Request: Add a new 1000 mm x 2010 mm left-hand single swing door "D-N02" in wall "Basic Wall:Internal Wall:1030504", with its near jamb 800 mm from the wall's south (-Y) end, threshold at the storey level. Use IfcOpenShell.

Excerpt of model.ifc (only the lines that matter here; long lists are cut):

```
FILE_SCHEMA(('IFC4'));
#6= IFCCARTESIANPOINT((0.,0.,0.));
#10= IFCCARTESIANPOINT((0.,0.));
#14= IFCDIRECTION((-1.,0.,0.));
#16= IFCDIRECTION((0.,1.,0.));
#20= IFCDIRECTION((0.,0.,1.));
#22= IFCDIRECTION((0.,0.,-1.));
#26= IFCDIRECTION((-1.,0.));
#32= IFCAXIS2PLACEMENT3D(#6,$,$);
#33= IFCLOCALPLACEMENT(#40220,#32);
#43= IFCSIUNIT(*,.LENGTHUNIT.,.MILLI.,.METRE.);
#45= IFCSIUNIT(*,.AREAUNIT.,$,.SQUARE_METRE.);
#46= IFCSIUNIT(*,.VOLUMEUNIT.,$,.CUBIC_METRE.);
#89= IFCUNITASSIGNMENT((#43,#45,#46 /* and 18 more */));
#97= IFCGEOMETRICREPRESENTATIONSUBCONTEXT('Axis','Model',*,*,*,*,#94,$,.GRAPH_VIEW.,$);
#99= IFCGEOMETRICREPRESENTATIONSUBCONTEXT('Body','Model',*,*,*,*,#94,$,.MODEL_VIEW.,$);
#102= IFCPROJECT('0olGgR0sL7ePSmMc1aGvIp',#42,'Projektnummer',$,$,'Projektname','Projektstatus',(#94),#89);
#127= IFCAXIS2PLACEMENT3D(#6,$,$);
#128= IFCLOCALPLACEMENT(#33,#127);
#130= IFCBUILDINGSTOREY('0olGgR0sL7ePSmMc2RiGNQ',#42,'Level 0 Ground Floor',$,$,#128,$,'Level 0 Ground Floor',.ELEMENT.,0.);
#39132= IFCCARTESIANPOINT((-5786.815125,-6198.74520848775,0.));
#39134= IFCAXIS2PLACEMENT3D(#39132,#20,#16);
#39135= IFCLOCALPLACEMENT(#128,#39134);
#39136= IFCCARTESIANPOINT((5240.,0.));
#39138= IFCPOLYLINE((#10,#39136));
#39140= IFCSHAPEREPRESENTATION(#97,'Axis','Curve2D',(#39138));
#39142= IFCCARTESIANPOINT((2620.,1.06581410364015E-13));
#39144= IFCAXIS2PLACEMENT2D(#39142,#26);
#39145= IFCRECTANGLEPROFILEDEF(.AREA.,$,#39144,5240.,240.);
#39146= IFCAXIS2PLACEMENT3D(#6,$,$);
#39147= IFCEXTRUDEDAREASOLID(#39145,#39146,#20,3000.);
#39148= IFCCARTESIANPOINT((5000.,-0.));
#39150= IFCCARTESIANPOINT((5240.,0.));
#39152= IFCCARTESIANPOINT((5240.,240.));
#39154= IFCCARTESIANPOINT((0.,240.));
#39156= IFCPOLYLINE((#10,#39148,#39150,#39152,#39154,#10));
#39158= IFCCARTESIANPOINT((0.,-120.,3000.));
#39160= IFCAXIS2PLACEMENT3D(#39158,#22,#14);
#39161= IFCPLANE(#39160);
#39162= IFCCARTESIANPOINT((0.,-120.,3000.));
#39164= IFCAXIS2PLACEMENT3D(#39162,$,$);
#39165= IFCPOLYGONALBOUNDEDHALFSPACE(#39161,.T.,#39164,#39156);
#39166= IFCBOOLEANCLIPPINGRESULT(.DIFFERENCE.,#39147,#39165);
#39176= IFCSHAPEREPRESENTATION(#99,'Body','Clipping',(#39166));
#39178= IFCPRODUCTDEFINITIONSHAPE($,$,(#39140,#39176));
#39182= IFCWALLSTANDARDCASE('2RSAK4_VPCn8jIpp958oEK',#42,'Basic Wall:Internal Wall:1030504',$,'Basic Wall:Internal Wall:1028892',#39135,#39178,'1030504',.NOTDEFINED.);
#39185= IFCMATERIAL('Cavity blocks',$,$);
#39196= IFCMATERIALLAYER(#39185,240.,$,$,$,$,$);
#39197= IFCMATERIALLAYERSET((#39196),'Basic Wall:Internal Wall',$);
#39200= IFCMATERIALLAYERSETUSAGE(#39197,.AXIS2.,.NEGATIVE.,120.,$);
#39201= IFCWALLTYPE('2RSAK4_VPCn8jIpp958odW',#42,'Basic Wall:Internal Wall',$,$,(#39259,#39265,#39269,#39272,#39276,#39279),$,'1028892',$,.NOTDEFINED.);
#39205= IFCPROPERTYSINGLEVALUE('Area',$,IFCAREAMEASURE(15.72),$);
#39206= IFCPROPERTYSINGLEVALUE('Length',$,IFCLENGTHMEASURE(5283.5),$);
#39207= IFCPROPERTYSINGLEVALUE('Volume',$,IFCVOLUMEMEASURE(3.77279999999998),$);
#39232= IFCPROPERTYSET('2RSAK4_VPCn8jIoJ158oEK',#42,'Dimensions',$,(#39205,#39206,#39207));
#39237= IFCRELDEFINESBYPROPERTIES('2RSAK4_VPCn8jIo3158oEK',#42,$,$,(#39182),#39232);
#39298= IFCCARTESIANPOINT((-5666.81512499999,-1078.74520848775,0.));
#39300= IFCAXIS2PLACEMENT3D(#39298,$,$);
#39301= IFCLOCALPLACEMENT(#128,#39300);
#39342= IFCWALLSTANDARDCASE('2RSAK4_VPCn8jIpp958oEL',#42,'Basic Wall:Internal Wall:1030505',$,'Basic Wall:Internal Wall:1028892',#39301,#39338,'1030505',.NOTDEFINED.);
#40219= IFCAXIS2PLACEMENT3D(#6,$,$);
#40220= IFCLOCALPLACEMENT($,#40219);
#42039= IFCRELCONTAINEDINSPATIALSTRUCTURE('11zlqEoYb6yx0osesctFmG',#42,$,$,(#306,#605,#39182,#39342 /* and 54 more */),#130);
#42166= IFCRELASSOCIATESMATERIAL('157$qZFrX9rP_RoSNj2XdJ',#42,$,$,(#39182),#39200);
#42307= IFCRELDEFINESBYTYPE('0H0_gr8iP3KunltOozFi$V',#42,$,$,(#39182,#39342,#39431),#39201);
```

```python
import numpy as np
import ifcopenshell
import ifcopenshell.api.feature
import ifcopenshell.api.geometry
import ifcopenshell.api.pset
import ifcopenshell.api.root
import ifcopenshell.api.spatial
import ifcopenshell.geom
import ifcopenshell.util.element
import ifcopenshell.util.placement
import ifcopenshell.util.representation
import ifcopenshell.util.shape
import ifcopenshell.util.unit

model = ifcopenshell.open("model.ifc")
unit_scale = ifcopenshell.util.unit.calculate_unit_scale(model)
area_scale = ifcopenshell.util.unit.calculate_unit_scale(model, "AREAUNIT")
volume_scale = ifcopenshell.util.unit.calculate_unit_scale(model, "VOLUMEUNIT")
settings = ifcopenshell.geom.settings()


def volume(element):
    """Net volume in cubic metres, openings subtracted."""
    shape = ifcopenshell.geom.create_shape(settings, element)
    return ifcopenshell.util.shape.get_volume(shape.geometry)


wall = model.by_guid("2RSAK4_VPCn8jIpp958oEK")
storey = ifcopenshell.util.element.get_container(wall, ifc_class="IfcBuildingStorey")
context = ifcopenshell.util.representation.get_context(model, "Model", "Body", "MODEL_VIEW")
before = volume(wall)

width, height, from_end, sill = 1, 2.01, 0.8, 0.0  # metres

# The wall runs along its own X axis, and the end named is its -X end.
wall_shape = ifcopenshell.geom.create_shape(settings, wall)
x, y, z = ifcopenshell.util.shape.get_vertices(wall_shape.geometry).T
start = x.min() + from_end
face, thickness = float(y.min()), float(y.max() - y.min())
wall_matrix = ifcopenshell.util.placement.get_local_placement(wall.ObjectPlacement)
level = ifcopenshell.util.placement.get_local_placement(storey.ObjectPlacement)[2, 3]


def in_wall(x, y):
    """Placement at x, y metres in the wall's axes, at sill height."""
    matrix = wall_matrix.copy()
    matrix[:, 3] = wall_matrix @ np.array([x / unit_scale, y / unit_scale, 0.0, 1.0])
    matrix[2, 3] = level + sill / unit_scale
    return matrix


# Opening: a box that overshoots both wall faces by 50 mm.
opening = ifcopenshell.api.root.create_entity(model, ifc_class="IfcOpeningElement", predefined_type="OPENING")
box = ifcopenshell.api.geometry.add_wall_representation(
    model, context=context, length=width, height=height, thickness=thickness + 0.1
)
ifcopenshell.api.geometry.assign_representation(model, product=opening, representation=box)
ifcopenshell.api.geometry.edit_object_placement(model, product=opening, matrix=in_wall(start, face - 0.05), is_si=False)
ifcopenshell.api.feature.add_feature(model, feature=opening, element=wall)

door = ifcopenshell.api.root.create_entity(model, ifc_class="IfcDoor", name="D-N02", predefined_type="DOOR")
door.OverallWidth, door.OverallHeight = width / unit_scale, height / unit_scale
door.OperationType = "SINGLE_SWING_LEFT"
body = ifcopenshell.api.geometry.add_door_representation(
    model,
    context=context,
    overall_width=door.OverallWidth,
    overall_height=door.OverallHeight,
    operation_type="SINGLE_SWING_LEFT",
    lining_properties={"LiningDepth": thickness / unit_scale, "ThresholdDepth": thickness / unit_scale},
)
ifcopenshell.api.geometry.assign_representation(model, product=door, representation=body)
ifcopenshell.api.spatial.assign_container(model, products=[door], relating_structure=storey)
ifcopenshell.api.feature.add_filling(model, opening=opening, element=door)

# The lining spans the wall, so the door starts at the wall face.
ifcopenshell.api.geometry.edit_object_placement(model, product=door, matrix=in_wall(start, face), is_si=False)

after = volume(wall)

# Update the wall's stored quantities.
pset = model.by_id(ifcopenshell.util.element.get_pset(wall, "Dimensions", should_inherit=False)["id"])
ifcopenshell.api.pset.edit_pset(model, pset=pset, properties={
    "Area": model.create_entity("IfcAreaMeasure", after / thickness / area_scale),
    "Volume": model.create_entity("IfcVolumeMeasure", after / volume_scale),
})

print(f"wall volume {before:.3f} -> {after:.3f} m3")

model.write("model-out.ifc")
```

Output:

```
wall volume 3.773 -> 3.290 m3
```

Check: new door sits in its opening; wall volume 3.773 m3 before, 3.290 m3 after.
